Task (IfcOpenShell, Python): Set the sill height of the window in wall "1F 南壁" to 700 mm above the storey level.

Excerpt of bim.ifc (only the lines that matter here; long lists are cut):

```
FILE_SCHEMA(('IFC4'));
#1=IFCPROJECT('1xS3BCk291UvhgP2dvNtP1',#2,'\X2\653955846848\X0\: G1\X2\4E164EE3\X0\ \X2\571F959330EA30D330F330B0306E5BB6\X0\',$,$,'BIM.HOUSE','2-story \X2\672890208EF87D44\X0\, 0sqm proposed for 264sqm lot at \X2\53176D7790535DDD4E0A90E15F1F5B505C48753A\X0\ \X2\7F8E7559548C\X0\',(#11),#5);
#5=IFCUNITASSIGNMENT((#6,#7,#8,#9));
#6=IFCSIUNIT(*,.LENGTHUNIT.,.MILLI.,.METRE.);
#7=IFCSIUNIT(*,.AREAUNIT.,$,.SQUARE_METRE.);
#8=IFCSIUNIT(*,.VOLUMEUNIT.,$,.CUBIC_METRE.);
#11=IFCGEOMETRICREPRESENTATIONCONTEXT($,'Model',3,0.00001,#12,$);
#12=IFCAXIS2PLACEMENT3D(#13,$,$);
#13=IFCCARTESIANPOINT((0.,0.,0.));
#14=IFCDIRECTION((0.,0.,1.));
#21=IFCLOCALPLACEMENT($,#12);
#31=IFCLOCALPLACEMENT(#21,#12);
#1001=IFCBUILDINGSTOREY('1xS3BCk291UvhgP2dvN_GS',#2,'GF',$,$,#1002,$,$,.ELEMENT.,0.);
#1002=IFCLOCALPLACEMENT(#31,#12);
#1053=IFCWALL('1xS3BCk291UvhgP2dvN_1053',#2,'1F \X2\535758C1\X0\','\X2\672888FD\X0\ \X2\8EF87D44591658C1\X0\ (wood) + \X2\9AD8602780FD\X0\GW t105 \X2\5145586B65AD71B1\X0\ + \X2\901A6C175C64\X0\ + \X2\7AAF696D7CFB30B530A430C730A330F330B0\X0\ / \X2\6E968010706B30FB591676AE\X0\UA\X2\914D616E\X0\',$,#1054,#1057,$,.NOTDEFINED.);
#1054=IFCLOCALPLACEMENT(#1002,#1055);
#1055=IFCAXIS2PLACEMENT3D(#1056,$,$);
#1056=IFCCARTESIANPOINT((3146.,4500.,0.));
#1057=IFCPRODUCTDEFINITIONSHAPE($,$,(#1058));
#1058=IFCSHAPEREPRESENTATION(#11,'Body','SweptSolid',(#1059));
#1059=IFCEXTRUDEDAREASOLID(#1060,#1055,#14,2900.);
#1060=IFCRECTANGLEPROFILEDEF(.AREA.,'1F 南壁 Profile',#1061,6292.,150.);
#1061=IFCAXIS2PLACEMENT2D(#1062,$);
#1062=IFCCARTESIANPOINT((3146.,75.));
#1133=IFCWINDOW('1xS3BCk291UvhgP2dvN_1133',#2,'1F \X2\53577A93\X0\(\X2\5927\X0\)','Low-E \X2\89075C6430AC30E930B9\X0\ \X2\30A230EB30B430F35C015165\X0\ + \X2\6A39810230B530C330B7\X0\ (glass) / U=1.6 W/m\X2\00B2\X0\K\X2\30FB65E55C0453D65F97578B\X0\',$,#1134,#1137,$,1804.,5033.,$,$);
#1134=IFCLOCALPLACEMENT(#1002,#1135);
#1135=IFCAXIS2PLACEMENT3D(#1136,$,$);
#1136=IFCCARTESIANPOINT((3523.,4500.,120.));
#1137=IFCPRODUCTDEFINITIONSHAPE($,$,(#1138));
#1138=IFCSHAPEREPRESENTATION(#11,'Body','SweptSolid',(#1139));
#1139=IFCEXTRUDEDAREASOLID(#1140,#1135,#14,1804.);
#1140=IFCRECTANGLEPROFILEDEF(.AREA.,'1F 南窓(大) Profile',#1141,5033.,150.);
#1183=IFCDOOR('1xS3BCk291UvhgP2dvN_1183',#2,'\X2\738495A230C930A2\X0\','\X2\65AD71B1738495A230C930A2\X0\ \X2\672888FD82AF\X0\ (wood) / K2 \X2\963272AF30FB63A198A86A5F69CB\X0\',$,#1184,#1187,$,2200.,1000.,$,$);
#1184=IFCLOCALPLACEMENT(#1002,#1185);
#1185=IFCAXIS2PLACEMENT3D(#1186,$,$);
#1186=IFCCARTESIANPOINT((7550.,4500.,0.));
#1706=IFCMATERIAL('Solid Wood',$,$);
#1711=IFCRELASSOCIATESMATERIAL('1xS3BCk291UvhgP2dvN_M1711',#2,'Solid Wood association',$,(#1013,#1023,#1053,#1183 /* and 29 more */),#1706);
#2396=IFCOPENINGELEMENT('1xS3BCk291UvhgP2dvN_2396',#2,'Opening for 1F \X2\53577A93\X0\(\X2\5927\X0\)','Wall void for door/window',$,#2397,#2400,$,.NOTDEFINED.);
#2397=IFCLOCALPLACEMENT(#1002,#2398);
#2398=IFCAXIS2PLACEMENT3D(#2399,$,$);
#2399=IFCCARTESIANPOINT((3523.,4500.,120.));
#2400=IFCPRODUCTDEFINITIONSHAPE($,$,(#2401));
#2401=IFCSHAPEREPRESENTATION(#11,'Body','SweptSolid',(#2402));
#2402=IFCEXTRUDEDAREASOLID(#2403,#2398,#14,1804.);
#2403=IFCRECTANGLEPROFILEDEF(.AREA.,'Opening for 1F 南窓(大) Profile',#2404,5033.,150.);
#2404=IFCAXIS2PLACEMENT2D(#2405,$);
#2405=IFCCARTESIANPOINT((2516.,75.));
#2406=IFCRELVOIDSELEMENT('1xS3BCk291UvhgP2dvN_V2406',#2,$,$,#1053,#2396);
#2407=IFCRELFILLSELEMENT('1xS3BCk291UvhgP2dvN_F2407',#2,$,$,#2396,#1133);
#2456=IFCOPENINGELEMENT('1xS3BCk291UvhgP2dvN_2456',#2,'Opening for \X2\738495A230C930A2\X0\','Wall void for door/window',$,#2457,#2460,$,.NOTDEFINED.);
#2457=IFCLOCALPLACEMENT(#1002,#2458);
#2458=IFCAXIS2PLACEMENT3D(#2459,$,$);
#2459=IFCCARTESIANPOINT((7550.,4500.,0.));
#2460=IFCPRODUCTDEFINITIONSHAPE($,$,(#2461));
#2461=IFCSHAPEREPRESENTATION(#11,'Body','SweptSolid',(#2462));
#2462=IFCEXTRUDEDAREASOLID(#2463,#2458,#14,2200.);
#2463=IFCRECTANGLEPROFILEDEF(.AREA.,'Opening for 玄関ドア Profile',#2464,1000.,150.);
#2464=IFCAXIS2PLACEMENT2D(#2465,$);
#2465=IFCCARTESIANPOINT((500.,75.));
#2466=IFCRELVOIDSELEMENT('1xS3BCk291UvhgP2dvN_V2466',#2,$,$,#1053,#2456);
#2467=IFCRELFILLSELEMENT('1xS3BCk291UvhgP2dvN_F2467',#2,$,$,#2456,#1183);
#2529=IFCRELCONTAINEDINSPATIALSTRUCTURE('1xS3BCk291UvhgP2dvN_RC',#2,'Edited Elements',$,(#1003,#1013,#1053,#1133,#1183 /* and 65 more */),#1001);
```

```python
import numpy as np
import ifcopenshell
import ifcopenshell.api.geometry
import ifcopenshell.geom
import ifcopenshell.util.element
import ifcopenshell.util.placement
import ifcopenshell.util.shape
import ifcopenshell.util.unit

model = ifcopenshell.open("bim.ifc")
unit_scale = ifcopenshell.util.unit.calculate_unit_scale(model)

window = model.by_id(1133)
opening = window.FillsVoids[0].RelatingOpeningElement
storey = ifcopenshell.util.element.get_container(window, ifc_class="IfcBuildingStorey")
level = ifcopenshell.util.placement.get_local_placement(storey.ObjectPlacement)[2, 3]

# The opening's origin need not be at the sill, so measure its lowest point.
shape = ifcopenshell.geom.create_shape(ifcopenshell.geom.settings(), opening)
bottom = ifcopenshell.util.shape.get_shape_bottom_elevation(shape, shape.geometry) / unit_scale
dz = level + 700.0 - bottom

shift = np.array([0.0, 0.0, dz])
# The window is not placed relative to its opening, so move both.
for product in (opening, window):
    matrix = ifcopenshell.util.placement.get_local_placement(product.ObjectPlacement)
    matrix[:3, 3] += shift
    ifcopenshell.api.geometry.edit_object_placement(model, product=product, matrix=matrix, is_si=False)

print(f"moved by {dz * unit_scale:+.3f} m")

model.write("bim_updated.ifc")
```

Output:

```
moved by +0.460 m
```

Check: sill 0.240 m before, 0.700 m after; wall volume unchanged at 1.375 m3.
